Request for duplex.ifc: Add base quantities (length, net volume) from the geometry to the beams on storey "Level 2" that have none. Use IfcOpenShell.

First a look at what the model holds.

```python
import ifcopenshell
import ifcopenshell.util.element
import ifcopenshell.util.unit

model = ifcopenshell.open("duplex.ifc")
print(model.schema)
for unit_type in ("LENGTHUNIT", "AREAUNIT", "VOLUMEUNIT"):
    print(unit_type, ifcopenshell.util.unit.calculate_unit_scale(model, unit_type))
storey = next(s for s in model.by_type("IfcBuildingStorey") if s.Name == "Level 2")
beams = [e for e in ifcopenshell.util.element.get_decomposition(storey) if e.is_a("IfcBeam")]
for e in sorted(beams, key=lambda e: e.id()):
    print(e.id(), e.is_a(), e.Name, list(ifcopenshell.util.element.get_psets(e, qtos_only=True)), sep=" | ")
```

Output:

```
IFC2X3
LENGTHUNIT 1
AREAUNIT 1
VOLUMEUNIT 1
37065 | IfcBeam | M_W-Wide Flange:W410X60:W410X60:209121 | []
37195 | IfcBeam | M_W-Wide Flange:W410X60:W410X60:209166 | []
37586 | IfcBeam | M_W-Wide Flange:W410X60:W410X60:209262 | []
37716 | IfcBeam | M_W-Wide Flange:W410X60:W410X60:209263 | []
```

```python
import ifcopenshell
import ifcopenshell.api.pset
import ifcopenshell.geom
import ifcopenshell.util.element
import ifcopenshell.util.shape
import ifcopenshell.util.unit

model = ifcopenshell.open("duplex.ifc")
unit_scale = ifcopenshell.util.unit.calculate_unit_scale(model)
volume_scale = ifcopenshell.util.unit.calculate_unit_scale(model, "VOLUMEUNIT")
settings = ifcopenshell.geom.settings()

storey = next(s for s in model.by_type("IfcBuildingStorey") if s.Name == "Level 2")
beams = [e for e in ifcopenshell.util.element.get_decomposition(storey) if e.is_a("IfcBeam")]

for e in sorted(beams, key=lambda e: e.id()):
    if ifcopenshell.util.element.get_psets(e, qtos_only=True, should_inherit=False):
        continue
    # Geometry comes back in metres, in the element's own axes.
    shape = ifcopenshell.geom.create_shape(settings, e)
    values = {
        "Length": ifcopenshell.util.shape.get_max_xyz(shape.geometry) / unit_scale,
        "NetVolume": ifcopenshell.util.shape.get_volume(shape.geometry) / volume_scale,
    }
    qto = ifcopenshell.api.pset.add_qto(model, product=e, name="BaseQuantities")
    ifcopenshell.api.pset.edit_qto(model, qto=qto, properties=values)
    print(e.id(), {k: round(v, 3) for k, v in values.items()})

model.write("duplex-out.ifc")
```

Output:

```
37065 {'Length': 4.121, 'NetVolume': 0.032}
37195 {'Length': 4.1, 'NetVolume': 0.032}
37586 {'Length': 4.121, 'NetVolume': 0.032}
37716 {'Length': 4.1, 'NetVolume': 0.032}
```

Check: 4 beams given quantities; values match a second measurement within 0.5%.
